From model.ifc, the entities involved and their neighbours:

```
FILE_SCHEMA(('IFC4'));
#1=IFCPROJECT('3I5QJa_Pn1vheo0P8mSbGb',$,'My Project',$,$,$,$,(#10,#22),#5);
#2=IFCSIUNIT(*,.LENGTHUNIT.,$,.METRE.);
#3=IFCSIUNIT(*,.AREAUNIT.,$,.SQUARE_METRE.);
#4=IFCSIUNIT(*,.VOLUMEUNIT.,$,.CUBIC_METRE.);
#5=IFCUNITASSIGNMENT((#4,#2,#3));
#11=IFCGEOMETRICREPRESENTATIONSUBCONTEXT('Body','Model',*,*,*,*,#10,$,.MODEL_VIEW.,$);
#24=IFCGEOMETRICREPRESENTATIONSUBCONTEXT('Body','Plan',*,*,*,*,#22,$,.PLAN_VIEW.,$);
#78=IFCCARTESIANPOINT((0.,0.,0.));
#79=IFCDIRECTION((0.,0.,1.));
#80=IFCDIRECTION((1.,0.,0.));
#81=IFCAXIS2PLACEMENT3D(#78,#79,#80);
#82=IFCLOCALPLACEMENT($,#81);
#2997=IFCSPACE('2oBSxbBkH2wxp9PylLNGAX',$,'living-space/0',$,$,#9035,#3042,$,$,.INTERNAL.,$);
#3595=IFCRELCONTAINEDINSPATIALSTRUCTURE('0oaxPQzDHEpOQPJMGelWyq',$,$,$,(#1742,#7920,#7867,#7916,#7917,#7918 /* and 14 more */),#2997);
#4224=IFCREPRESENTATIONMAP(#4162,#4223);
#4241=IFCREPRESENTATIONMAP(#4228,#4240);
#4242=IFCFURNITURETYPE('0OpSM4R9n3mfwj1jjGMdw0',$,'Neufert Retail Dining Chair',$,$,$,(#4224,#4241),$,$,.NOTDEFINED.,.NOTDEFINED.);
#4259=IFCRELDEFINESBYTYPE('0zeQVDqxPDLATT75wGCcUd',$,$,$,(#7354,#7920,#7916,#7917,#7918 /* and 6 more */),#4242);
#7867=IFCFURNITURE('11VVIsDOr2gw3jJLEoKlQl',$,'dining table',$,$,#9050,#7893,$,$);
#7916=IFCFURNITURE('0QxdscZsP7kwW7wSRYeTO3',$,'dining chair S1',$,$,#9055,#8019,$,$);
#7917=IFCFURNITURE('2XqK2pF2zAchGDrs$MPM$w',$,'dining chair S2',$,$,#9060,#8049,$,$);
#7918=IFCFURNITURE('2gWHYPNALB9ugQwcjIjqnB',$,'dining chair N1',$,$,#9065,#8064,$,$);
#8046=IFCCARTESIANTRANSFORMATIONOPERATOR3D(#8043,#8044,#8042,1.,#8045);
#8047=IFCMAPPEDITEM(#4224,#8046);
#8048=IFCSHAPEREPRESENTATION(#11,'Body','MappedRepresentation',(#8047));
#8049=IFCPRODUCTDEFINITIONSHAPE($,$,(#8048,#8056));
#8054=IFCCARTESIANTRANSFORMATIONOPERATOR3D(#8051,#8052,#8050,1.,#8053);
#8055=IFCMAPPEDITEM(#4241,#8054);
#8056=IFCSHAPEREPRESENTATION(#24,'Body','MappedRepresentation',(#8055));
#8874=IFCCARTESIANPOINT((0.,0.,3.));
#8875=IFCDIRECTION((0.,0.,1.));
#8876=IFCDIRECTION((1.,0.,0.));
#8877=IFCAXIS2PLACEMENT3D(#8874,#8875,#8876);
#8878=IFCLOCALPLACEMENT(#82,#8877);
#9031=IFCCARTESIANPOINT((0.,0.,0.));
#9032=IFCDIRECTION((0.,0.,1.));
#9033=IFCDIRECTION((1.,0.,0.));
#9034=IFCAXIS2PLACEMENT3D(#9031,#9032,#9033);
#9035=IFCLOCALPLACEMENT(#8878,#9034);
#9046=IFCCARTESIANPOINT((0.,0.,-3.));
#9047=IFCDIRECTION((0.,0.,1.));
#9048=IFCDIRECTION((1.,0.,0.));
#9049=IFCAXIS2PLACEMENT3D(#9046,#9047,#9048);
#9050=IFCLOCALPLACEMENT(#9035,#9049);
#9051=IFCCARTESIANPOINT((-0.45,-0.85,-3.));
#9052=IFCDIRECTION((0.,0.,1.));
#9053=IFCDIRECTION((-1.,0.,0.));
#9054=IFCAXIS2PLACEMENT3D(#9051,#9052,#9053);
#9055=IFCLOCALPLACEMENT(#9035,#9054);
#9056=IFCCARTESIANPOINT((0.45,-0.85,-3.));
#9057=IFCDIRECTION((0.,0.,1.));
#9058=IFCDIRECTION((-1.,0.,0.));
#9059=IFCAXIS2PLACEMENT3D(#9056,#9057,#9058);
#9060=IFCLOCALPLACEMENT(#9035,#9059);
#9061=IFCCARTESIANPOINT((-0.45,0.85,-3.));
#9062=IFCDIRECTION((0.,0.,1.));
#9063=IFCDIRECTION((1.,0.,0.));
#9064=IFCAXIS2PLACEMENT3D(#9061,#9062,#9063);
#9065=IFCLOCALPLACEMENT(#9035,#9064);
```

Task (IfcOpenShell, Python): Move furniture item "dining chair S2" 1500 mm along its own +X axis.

```python
import ifcopenshell
import ifcopenshell.api.geometry
import ifcopenshell.util.placement
import ifcopenshell.util.unit

model = ifcopenshell.open("model.ifc")
unit_scale = ifcopenshell.util.unit.calculate_unit_scale(model)

item = model.by_id(7917)
matrix = ifcopenshell.util.placement.get_local_placement(item.ObjectPlacement)
matrix[:3, 3] += matrix[:3, 0] * 1.5 / unit_scale
ifcopenshell.api.geometry.edit_object_placement(model, product=item, matrix=matrix, is_si=False)

print(ifcopenshell.util.placement.get_local_placement(item.ObjectPlacement).round(3) + 0.0)

model.write("model-out.ifc")
```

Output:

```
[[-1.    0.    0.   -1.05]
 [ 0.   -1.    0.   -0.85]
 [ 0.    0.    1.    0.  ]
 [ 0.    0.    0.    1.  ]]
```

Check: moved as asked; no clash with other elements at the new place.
